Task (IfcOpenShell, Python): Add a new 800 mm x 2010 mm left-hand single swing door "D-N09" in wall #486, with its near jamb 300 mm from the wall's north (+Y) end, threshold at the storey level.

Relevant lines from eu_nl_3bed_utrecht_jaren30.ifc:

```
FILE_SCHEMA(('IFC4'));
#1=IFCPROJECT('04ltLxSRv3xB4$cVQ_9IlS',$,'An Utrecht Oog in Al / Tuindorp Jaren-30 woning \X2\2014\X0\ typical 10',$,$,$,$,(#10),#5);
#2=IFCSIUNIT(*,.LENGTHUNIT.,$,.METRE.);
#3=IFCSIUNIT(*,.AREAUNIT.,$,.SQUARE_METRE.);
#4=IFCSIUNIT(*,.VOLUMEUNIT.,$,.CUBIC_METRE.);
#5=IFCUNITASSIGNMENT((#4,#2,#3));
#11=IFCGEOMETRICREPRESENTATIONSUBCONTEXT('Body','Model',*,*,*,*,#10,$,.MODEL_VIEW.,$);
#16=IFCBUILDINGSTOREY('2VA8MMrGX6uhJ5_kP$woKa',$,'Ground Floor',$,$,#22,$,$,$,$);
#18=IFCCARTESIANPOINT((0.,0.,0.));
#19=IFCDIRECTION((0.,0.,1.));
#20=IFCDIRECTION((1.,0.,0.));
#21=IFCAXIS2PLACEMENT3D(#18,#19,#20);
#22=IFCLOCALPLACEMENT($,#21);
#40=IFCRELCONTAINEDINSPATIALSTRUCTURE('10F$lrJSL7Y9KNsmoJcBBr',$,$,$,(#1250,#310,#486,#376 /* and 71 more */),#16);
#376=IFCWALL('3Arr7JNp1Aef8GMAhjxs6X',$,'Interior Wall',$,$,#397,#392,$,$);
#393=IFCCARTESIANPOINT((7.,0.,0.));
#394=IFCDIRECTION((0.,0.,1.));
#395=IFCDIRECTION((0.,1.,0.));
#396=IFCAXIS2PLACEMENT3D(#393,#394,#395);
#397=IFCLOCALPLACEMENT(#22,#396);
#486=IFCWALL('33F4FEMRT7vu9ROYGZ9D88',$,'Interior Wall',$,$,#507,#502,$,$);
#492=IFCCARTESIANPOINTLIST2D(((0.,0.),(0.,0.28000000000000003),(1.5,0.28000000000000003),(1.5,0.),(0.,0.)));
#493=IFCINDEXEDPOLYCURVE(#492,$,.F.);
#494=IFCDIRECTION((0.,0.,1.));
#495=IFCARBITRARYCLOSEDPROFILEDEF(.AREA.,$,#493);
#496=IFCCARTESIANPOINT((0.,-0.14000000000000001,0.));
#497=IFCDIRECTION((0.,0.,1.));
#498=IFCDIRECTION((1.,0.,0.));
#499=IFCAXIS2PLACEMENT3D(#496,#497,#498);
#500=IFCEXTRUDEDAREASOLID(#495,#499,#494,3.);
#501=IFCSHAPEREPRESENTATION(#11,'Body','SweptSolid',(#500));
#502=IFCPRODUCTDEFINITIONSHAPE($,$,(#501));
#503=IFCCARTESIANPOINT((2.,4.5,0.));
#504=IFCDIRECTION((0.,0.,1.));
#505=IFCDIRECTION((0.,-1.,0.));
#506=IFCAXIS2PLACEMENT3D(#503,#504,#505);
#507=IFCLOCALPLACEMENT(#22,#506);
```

```python
import numpy as np
import ifcopenshell
import ifcopenshell.api.feature
import ifcopenshell.api.geometry
import ifcopenshell.api.root
import ifcopenshell.api.spatial
import ifcopenshell.geom
import ifcopenshell.util.element
import ifcopenshell.util.placement
import ifcopenshell.util.representation
import ifcopenshell.util.shape
import ifcopenshell.util.unit

model = ifcopenshell.open("eu_nl_3bed_utrecht_jaren30.ifc")
unit_scale = ifcopenshell.util.unit.calculate_unit_scale(model)
settings = ifcopenshell.geom.settings()


def volume(element):
    """Net volume in cubic metres, openings subtracted."""
    shape = ifcopenshell.geom.create_shape(settings, element)
    return ifcopenshell.util.shape.get_volume(shape.geometry)


wall = model.by_guid("33F4FEMRT7vu9ROYGZ9D88")
storey = ifcopenshell.util.element.get_container(wall, ifc_class="IfcBuildingStorey")
context = ifcopenshell.util.representation.get_context(model, "Model", "Body", "MODEL_VIEW")
before = volume(wall)

width, height, from_end, sill = 0.8, 2.01, 0.3, 0.0  # metres

# The wall runs along its own X axis, and the end named is its -X end.
wall_shape = ifcopenshell.geom.create_shape(settings, wall)
x, y, z = ifcopenshell.util.shape.get_vertices(wall_shape.geometry).T
start = x.min() + from_end
face, thickness = float(y.min()), float(y.max() - y.min())
wall_matrix = ifcopenshell.util.placement.get_local_placement(wall.ObjectPlacement)
level = ifcopenshell.util.placement.get_local_placement(storey.ObjectPlacement)[2, 3]


def in_wall(x, y):
    """Placement at x, y metres in the wall's axes, at sill height."""
    matrix = wall_matrix.copy()
    matrix[:, 3] = wall_matrix @ np.array([x / unit_scale, y / unit_scale, 0.0, 1.0])
    matrix[2, 3] = level + sill / unit_scale
    return matrix


# Opening: a box that overshoots both wall faces by 50 mm.
opening = ifcopenshell.api.root.create_entity(model, ifc_class="IfcOpeningElement", predefined_type="OPENING")
box = ifcopenshell.api.geometry.add_wall_representation(
    model, context=context, length=width, height=height, thickness=thickness + 0.1
)
ifcopenshell.api.geometry.assign_representation(model, product=opening, representation=box)
ifcopenshell.api.geometry.edit_object_placement(model, product=opening, matrix=in_wall(start, face - 0.05), is_si=False)
ifcopenshell.api.feature.add_feature(model, feature=opening, element=wall)

door = ifcopenshell.api.root.create_entity(model, ifc_class="IfcDoor", name="D-N09", predefined_type="DOOR")
door.OverallWidth, door.OverallHeight = width / unit_scale, height / unit_scale
door.OperationType = "SINGLE_SWING_LEFT"
body = ifcopenshell.api.geometry.add_door_representation(
    model,
    context=context,
    overall_width=door.OverallWidth,
    overall_height=door.OverallHeight,
    operation_type="SINGLE_SWING_LEFT",
    lining_properties={"LiningDepth": thickness / unit_scale, "ThresholdDepth": thickness / unit_scale},
)
ifcopenshell.api.geometry.assign_representation(model, product=door, representation=body)
ifcopenshell.api.spatial.assign_container(model, products=[door], relating_structure=storey)
ifcopenshell.api.feature.add_filling(model, opening=opening, element=door)

# The lining spans the wall, so the door starts at the wall face.
ifcopenshell.api.geometry.edit_object_placement(model, product=door, matrix=in_wall(start, face), is_si=False)

after = volume(wall)

print(f"wall volume {before:.3f} -> {after:.3f} m3")

model.write("eu_nl_3bed_utrecht_jaren30_rev.ifc")
```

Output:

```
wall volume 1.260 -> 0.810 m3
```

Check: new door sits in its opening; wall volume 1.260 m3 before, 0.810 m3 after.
